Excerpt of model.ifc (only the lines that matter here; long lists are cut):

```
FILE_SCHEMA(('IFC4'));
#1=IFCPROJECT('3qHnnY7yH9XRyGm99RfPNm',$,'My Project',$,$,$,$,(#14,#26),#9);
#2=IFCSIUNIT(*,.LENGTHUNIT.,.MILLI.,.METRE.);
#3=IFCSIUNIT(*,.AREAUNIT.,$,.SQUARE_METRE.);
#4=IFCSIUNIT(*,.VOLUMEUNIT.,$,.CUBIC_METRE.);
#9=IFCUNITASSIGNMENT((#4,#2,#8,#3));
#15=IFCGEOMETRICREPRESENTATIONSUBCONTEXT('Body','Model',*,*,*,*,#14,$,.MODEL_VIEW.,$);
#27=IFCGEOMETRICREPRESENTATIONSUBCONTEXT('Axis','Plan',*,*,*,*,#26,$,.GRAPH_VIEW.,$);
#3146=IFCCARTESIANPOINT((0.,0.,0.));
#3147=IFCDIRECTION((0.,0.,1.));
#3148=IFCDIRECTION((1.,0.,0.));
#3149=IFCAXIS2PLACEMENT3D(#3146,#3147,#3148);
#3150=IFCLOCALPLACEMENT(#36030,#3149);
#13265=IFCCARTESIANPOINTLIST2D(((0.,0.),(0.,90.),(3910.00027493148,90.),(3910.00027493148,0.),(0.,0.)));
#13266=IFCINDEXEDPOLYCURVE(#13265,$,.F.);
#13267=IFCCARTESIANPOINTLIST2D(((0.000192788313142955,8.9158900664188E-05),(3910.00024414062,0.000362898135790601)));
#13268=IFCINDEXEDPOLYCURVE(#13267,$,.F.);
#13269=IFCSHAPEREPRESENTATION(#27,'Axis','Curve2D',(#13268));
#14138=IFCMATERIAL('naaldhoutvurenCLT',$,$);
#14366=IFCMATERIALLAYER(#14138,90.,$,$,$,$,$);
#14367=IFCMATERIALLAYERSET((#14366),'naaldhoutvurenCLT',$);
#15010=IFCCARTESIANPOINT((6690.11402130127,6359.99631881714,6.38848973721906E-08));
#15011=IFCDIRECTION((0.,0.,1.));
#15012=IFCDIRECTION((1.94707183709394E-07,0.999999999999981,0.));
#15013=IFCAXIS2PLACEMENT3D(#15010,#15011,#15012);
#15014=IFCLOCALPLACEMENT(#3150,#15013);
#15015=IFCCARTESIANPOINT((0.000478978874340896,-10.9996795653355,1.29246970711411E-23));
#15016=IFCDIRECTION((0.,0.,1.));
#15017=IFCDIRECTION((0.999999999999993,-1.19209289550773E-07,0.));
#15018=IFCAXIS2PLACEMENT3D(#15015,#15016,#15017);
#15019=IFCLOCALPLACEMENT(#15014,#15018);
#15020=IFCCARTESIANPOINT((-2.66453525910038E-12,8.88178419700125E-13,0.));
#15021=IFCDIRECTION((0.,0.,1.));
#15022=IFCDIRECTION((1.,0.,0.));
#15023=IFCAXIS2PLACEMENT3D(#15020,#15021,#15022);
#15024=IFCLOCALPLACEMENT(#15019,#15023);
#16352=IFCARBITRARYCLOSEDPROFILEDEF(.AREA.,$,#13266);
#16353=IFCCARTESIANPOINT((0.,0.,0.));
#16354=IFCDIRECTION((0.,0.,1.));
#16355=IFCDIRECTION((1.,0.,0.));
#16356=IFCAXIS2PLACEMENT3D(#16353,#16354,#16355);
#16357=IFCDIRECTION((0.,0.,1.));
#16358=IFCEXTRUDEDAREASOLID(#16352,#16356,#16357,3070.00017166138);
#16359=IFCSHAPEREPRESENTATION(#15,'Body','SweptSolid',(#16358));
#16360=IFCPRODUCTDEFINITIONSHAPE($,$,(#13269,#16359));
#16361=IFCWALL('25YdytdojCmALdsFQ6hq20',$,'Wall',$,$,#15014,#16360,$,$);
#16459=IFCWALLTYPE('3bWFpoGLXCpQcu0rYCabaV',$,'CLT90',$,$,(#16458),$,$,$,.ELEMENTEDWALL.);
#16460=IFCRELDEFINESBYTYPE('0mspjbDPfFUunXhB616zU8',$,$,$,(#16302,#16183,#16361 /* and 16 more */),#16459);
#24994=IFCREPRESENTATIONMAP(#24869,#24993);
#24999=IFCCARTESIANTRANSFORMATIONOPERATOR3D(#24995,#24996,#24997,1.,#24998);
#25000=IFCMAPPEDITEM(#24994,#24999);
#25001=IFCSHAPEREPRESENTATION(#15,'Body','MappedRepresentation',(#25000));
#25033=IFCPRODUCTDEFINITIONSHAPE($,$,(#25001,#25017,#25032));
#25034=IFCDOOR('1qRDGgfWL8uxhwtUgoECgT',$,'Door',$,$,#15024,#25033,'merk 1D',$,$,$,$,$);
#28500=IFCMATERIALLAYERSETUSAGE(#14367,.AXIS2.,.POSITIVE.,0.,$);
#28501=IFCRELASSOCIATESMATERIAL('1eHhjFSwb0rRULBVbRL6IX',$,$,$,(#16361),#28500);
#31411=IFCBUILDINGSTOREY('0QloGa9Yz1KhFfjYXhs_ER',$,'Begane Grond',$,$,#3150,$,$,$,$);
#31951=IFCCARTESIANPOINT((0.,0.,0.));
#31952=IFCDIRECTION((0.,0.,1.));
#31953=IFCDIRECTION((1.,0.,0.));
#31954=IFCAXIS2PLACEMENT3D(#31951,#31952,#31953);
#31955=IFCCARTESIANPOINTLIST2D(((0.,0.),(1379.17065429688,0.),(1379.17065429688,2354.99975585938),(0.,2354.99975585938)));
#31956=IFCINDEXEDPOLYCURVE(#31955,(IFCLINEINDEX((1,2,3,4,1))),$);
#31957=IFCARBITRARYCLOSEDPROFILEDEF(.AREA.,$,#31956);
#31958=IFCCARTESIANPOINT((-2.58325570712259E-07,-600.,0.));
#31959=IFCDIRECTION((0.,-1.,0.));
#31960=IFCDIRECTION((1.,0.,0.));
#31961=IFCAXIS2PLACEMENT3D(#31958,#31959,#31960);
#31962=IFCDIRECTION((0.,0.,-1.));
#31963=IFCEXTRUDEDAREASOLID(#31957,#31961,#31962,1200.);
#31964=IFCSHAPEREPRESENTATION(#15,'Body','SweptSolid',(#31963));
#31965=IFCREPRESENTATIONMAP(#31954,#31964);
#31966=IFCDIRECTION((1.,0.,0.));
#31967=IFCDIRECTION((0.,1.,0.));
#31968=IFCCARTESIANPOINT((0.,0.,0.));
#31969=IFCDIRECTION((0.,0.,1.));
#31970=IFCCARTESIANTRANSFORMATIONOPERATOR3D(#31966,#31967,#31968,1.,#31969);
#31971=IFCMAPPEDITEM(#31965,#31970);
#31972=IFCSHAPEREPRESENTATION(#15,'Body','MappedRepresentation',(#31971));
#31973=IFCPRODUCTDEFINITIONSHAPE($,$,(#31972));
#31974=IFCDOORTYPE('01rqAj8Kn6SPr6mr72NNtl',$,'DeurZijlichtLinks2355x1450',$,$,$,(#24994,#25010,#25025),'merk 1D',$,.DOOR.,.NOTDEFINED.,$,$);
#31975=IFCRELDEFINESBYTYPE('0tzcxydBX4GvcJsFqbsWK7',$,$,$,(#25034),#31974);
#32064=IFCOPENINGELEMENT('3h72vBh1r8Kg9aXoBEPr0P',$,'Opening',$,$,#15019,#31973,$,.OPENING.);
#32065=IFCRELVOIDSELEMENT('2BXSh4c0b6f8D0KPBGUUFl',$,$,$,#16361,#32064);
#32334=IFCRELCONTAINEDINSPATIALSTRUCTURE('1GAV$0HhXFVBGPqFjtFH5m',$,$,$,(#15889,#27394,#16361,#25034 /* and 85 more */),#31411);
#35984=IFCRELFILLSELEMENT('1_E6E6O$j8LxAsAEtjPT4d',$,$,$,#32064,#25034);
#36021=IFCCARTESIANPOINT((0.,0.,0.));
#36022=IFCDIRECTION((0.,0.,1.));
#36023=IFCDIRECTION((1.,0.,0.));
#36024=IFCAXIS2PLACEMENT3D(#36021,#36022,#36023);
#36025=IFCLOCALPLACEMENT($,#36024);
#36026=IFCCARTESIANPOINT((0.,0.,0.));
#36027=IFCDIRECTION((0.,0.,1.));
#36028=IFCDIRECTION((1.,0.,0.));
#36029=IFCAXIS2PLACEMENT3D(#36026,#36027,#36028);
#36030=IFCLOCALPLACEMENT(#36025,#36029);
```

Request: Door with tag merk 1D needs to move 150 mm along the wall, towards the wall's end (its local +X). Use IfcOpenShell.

```python
import ifcopenshell
import ifcopenshell.api.geometry
import ifcopenshell.util.placement

model = ifcopenshell.open("model.ifc")

door = model.by_guid("1qRDGgfWL8uxhwtUgoECgT")
opening = door.FillsVoids[0].RelatingOpeningElement
wall = opening.VoidsElements[0].RelatingBuildingElement

wall_matrix = ifcopenshell.util.placement.get_local_placement(wall.ObjectPlacement)
shift = wall_matrix[:3, 0] * 150.0
before = ifcopenshell.util.placement.get_local_placement(door.ObjectPlacement)[:3, 3].copy()

# The door is placed relative to its opening, so it follows when the opening moves.
matrix = ifcopenshell.util.placement.get_local_placement(opening.ObjectPlacement)
matrix[:3, 3] += shift
ifcopenshell.api.geometry.edit_object_placement(
    model, product=opening, matrix=matrix, is_si=False, should_transform_children=True
)

after = ifcopenshell.util.placement.get_local_placement(door.ObjectPlacement)[:3, 3]
print("door moved by", (after - before).round(3) + 0.0)

model.write("model-out.ifc")
```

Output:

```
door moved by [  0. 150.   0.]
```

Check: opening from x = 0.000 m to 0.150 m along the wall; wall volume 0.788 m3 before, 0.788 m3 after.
